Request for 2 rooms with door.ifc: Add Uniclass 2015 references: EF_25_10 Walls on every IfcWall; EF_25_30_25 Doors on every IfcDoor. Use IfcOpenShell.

First a look at what the model holds.

```python
import ifcopenshell

model = ifcopenshell.open("2 rooms with door.ifc")
print(model.schema)
print("classifications:", [c.Name for c in model.by_type("IfcClassification")])
for ifc_class in ("IfcDoor", "IfcRoof", "IfcStair", "IfcWall", "IfcWindow"):
    print(ifc_class, len(model.by_type(ifc_class)))
```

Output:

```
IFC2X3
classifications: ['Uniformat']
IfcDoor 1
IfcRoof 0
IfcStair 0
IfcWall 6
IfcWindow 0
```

```python
import ifcopenshell
import ifcopenshell.api.classification

model = ifcopenshell.open("2 rooms with door.ifc")

# IFC2X3 requires Source and Edition and has no link from the project to the system.
system = model.create_entity("IfcClassification", Source="NBS", Edition="2015", Name="Uniclass 2015")

codes = {
    "IfcWall": ("EF_25_10", "Walls"),
    "IfcDoor": ("EF_25_30_25", "Doors"),
}
for ifc_class, (code, name) in codes.items():
    products = model.by_type(ifc_class)
    ifcopenshell.api.classification.add_reference(
        model, products=products, classification=system, identification=code, name=name
    )
    print(code, len(products))

model.write("2 rooms with door_updated.ifc")
```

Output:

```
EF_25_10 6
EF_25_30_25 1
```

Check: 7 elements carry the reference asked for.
